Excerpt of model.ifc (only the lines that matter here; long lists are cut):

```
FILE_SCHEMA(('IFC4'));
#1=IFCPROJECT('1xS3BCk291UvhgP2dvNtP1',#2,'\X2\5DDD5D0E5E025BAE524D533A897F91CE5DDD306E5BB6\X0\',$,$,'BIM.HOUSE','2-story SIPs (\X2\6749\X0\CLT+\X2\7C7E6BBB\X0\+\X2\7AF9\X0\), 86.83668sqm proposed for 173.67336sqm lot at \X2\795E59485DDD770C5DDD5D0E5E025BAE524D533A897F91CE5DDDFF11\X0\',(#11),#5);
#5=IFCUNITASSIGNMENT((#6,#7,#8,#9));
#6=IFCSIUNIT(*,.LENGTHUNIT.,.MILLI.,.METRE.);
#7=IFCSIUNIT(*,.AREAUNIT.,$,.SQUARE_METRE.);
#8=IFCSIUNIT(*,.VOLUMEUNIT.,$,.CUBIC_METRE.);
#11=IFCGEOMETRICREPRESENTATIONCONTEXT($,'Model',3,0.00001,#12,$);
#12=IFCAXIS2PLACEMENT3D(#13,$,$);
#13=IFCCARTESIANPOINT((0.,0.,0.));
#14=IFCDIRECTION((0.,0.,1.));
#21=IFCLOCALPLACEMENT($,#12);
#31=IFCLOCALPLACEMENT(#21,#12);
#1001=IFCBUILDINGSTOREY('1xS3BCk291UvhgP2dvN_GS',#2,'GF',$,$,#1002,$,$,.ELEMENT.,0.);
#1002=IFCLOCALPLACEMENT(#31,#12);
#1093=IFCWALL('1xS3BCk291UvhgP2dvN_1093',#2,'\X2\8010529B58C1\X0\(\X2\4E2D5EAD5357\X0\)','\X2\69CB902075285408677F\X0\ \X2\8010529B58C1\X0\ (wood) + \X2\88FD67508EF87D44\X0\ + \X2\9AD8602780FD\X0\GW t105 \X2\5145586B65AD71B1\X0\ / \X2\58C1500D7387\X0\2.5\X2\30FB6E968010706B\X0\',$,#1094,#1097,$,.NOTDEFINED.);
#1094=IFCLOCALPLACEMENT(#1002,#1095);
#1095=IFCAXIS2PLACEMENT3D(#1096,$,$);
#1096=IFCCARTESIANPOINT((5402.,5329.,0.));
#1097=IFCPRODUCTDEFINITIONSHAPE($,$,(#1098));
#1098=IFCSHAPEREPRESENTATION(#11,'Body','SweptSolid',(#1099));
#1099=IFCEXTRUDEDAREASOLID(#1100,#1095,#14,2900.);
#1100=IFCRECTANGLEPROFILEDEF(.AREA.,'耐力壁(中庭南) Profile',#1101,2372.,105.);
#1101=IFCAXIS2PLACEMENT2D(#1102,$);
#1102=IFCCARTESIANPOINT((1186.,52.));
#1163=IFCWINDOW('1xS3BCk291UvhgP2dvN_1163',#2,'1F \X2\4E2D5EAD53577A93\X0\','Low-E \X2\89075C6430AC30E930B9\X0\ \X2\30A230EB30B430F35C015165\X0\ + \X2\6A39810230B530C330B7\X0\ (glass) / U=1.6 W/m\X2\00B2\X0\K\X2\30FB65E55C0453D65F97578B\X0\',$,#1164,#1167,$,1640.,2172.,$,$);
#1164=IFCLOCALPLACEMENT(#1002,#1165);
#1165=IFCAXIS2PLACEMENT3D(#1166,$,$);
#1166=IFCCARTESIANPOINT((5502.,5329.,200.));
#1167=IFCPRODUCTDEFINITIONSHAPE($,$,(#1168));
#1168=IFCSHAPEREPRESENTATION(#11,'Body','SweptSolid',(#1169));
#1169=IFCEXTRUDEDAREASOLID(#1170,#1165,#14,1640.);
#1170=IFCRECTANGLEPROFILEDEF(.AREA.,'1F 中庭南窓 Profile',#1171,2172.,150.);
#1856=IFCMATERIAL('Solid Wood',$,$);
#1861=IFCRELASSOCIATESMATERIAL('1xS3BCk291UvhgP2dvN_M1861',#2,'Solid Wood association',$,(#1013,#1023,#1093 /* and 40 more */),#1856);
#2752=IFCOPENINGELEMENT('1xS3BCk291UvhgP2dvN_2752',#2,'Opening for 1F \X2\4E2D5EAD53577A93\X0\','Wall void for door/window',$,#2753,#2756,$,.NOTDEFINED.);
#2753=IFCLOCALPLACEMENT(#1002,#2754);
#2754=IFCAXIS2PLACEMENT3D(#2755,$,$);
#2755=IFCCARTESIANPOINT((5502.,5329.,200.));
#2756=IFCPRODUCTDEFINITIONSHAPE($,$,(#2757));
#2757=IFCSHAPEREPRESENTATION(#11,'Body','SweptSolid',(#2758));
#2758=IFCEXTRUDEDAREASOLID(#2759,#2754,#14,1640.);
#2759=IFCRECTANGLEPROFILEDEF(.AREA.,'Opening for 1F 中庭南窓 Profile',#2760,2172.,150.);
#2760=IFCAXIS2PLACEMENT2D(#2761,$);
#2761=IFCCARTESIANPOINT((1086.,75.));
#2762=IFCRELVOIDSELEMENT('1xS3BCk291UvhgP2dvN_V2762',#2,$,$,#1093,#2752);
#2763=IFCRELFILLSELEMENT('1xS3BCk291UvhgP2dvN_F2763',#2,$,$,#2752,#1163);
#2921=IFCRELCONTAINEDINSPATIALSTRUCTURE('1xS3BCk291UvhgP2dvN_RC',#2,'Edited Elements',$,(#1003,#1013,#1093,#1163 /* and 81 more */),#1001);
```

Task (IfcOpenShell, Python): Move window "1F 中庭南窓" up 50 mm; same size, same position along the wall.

```python
import numpy as np
import ifcopenshell
import ifcopenshell.api.geometry
import ifcopenshell.util.placement
import ifcopenshell.util.unit

model = ifcopenshell.open("model.ifc")
unit_scale = ifcopenshell.util.unit.calculate_unit_scale(model)

window = model.by_guid("1xS3BCk291UvhgP2dvN_1163")
opening = window.FillsVoids[0].RelatingOpeningElement
dz = 0.05 / unit_scale

shift = np.array([0.0, 0.0, dz])
# The window is not placed relative to its opening, so move both.
for product in (opening, window):
    matrix = ifcopenshell.util.placement.get_local_placement(product.ObjectPlacement)
    matrix[:3, 3] += shift
    ifcopenshell.api.geometry.edit_object_placement(model, product=product, matrix=matrix, is_si=False)

print(f"moved by {dz * unit_scale:+.3f} m")

model.write("model_edited.ifc")
```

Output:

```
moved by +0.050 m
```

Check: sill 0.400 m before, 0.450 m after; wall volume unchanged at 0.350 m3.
